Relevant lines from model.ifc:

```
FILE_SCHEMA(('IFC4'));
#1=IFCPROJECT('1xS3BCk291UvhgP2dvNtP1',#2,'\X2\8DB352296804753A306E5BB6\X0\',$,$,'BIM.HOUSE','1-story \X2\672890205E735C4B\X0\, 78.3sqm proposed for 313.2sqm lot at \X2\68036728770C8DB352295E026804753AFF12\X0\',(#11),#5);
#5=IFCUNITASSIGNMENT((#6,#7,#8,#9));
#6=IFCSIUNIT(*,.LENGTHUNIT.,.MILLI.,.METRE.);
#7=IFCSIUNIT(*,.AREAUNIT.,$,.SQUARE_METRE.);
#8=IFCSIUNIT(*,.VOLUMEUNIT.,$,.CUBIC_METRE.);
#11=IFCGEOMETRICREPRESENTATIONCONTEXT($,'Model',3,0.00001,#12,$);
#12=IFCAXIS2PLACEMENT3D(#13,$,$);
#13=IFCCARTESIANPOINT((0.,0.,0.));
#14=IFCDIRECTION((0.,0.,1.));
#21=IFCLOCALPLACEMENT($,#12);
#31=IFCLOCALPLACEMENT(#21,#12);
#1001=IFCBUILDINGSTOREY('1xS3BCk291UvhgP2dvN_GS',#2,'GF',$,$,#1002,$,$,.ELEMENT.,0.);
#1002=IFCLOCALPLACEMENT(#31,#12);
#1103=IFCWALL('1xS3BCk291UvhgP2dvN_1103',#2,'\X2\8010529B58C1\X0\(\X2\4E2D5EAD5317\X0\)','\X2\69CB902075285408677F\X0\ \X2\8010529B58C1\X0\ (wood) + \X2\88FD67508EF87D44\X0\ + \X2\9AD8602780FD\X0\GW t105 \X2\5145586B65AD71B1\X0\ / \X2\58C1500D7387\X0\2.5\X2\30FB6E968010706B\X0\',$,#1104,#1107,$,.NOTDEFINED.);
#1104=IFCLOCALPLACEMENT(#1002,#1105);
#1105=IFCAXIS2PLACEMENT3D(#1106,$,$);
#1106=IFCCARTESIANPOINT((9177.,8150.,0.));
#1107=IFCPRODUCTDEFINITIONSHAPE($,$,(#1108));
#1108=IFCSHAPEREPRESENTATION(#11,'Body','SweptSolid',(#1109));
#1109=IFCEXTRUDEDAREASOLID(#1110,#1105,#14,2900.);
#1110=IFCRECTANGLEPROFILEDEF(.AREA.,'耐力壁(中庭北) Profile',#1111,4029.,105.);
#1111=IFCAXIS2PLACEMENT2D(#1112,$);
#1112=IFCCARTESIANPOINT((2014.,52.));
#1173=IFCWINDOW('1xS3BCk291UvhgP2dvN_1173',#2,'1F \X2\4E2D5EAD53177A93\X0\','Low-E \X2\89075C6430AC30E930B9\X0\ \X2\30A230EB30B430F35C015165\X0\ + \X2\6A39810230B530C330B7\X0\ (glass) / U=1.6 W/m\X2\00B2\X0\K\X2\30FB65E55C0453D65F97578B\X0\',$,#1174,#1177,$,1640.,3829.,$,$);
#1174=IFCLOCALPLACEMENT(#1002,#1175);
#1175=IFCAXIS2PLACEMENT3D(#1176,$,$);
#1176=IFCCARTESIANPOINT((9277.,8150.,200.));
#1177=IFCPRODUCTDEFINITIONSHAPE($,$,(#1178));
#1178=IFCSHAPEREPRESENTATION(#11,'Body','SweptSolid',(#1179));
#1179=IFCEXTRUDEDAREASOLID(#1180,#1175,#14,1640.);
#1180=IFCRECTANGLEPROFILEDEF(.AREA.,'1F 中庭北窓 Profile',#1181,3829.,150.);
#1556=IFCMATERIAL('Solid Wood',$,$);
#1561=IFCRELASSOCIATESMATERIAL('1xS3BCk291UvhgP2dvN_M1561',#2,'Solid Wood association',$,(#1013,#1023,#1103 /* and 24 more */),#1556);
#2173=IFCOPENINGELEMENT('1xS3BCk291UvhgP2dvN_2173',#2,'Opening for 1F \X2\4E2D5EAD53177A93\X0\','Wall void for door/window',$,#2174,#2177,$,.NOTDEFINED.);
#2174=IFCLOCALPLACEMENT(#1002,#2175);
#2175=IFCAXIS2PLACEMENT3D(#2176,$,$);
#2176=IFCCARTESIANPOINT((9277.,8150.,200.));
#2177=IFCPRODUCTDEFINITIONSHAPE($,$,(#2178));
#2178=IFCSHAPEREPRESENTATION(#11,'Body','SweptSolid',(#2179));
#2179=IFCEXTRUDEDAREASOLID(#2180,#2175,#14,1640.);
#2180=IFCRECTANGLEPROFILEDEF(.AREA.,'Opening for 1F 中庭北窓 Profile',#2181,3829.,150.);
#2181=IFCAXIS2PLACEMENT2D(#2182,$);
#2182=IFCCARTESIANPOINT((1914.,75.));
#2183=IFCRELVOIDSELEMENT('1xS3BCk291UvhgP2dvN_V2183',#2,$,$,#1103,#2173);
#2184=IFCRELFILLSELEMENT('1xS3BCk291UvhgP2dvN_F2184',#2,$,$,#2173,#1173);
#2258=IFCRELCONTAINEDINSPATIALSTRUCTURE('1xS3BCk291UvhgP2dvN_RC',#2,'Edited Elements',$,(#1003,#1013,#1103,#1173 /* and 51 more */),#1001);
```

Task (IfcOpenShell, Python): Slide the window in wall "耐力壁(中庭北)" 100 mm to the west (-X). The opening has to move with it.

```python
import ifcopenshell
import ifcopenshell.api.geometry
import ifcopenshell.util.placement
import ifcopenshell.util.unit

model = ifcopenshell.open("model.ifc")
unit_scale = ifcopenshell.util.unit.calculate_unit_scale(model)

window = model.by_guid("1xS3BCk291UvhgP2dvN_1173")
opening = window.FillsVoids[0].RelatingOpeningElement
wall = opening.VoidsElements[0].RelatingBuildingElement

wall_matrix = ifcopenshell.util.placement.get_local_placement(wall.ObjectPlacement)
shift = wall_matrix[:3, 0] * -0.1 / unit_scale
before = ifcopenshell.util.placement.get_local_placement(window.ObjectPlacement)[:3, 3].copy()

# The window is not placed relative to its opening, so move both.
for product in (opening, window):
    matrix = ifcopenshell.util.placement.get_local_placement(product.ObjectPlacement)
    matrix[:3, 3] += shift
    ifcopenshell.api.geometry.edit_object_placement(model, product=product, matrix=matrix, is_si=False)

after = ifcopenshell.util.placement.get_local_placement(window.ObjectPlacement)[:3, 3]
print("window moved by", (after - before).round(3) + 0.0)

model.write("model_edited.ifc")
```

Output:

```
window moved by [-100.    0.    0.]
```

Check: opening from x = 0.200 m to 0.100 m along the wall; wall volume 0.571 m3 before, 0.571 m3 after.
